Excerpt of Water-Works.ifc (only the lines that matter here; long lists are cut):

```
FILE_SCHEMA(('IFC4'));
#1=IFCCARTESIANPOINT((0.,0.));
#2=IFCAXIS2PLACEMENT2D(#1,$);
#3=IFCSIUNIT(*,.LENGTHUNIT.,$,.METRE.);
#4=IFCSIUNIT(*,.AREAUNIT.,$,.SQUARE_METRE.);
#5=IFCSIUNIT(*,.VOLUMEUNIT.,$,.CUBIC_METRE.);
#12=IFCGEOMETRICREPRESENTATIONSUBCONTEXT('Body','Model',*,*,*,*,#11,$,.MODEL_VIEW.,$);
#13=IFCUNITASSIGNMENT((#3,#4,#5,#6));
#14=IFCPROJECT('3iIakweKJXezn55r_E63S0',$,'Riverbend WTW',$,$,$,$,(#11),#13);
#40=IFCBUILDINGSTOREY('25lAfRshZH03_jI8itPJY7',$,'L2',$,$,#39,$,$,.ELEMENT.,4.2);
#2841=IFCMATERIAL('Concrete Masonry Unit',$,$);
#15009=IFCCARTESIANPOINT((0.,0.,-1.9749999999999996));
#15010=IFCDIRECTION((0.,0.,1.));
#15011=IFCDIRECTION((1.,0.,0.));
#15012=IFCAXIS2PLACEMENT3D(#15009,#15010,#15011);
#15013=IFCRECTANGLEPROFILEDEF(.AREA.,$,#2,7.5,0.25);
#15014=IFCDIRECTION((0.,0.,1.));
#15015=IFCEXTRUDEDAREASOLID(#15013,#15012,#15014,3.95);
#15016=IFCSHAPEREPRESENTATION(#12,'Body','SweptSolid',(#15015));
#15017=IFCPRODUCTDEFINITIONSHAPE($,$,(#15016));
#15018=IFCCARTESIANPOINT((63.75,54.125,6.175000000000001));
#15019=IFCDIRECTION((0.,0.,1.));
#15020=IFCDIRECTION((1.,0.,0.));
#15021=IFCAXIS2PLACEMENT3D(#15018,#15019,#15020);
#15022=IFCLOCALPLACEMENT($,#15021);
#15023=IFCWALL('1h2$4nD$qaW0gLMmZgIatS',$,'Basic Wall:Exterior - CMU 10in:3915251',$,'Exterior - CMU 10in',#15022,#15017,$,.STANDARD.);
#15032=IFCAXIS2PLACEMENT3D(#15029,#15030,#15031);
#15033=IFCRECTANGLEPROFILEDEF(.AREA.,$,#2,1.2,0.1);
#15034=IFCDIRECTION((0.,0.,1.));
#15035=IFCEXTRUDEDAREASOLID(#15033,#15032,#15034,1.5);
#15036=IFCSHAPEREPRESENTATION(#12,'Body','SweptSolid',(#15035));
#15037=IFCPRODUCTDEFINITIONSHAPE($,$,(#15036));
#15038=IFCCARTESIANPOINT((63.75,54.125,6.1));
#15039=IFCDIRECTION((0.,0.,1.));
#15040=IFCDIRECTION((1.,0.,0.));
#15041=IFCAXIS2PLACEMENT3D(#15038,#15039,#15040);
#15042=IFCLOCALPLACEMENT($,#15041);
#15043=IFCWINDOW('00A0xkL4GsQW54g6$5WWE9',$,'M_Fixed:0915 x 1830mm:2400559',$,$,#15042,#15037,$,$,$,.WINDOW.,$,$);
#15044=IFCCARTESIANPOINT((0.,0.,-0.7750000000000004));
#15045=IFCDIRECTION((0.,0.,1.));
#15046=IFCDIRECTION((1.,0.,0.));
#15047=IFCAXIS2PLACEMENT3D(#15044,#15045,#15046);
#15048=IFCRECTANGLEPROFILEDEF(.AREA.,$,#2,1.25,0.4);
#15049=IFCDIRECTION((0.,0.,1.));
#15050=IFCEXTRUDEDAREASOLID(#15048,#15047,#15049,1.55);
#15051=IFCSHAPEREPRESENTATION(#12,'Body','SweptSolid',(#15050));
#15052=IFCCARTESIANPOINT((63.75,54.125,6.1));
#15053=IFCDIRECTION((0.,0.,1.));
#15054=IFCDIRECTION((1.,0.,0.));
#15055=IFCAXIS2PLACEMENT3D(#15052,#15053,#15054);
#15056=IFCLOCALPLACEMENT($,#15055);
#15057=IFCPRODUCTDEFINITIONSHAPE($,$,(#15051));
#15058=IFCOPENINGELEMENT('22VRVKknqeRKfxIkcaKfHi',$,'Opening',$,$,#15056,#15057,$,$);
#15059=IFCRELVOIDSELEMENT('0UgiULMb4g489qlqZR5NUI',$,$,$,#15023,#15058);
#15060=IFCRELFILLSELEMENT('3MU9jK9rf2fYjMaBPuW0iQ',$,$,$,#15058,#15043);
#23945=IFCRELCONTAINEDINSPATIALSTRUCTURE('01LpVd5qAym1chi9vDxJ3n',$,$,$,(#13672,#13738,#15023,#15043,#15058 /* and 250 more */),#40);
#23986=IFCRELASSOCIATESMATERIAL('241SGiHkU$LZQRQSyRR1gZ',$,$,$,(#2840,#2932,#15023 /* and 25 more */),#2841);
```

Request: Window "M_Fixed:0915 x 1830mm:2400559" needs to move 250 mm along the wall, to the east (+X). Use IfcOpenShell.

```python
import ifcopenshell
import ifcopenshell.api.geometry
import ifcopenshell.util.placement

model = ifcopenshell.open("Water-Works.ifc")

window = model.by_id(15043)
opening = window.FillsVoids[0].RelatingOpeningElement
wall = opening.VoidsElements[0].RelatingBuildingElement

wall_matrix = ifcopenshell.util.placement.get_local_placement(wall.ObjectPlacement)
shift = wall_matrix[:3, 0] * 0.25
before = ifcopenshell.util.placement.get_local_placement(window.ObjectPlacement)[:3, 3].copy()

# The window is not placed relative to its opening, so move both.
for product in (opening, window):
    matrix = ifcopenshell.util.placement.get_local_placement(product.ObjectPlacement)
    matrix[:3, 3] += shift
    ifcopenshell.api.geometry.edit_object_placement(model, product=product, matrix=matrix, is_si=False)

after = ifcopenshell.util.placement.get_local_placement(window.ObjectPlacement)[:3, 3]
print("window moved by", (after - before).round(3) + 0.0)

model.write("Water-Works-out.ifc")
```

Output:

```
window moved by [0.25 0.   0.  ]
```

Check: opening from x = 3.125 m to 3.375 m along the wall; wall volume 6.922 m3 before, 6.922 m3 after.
